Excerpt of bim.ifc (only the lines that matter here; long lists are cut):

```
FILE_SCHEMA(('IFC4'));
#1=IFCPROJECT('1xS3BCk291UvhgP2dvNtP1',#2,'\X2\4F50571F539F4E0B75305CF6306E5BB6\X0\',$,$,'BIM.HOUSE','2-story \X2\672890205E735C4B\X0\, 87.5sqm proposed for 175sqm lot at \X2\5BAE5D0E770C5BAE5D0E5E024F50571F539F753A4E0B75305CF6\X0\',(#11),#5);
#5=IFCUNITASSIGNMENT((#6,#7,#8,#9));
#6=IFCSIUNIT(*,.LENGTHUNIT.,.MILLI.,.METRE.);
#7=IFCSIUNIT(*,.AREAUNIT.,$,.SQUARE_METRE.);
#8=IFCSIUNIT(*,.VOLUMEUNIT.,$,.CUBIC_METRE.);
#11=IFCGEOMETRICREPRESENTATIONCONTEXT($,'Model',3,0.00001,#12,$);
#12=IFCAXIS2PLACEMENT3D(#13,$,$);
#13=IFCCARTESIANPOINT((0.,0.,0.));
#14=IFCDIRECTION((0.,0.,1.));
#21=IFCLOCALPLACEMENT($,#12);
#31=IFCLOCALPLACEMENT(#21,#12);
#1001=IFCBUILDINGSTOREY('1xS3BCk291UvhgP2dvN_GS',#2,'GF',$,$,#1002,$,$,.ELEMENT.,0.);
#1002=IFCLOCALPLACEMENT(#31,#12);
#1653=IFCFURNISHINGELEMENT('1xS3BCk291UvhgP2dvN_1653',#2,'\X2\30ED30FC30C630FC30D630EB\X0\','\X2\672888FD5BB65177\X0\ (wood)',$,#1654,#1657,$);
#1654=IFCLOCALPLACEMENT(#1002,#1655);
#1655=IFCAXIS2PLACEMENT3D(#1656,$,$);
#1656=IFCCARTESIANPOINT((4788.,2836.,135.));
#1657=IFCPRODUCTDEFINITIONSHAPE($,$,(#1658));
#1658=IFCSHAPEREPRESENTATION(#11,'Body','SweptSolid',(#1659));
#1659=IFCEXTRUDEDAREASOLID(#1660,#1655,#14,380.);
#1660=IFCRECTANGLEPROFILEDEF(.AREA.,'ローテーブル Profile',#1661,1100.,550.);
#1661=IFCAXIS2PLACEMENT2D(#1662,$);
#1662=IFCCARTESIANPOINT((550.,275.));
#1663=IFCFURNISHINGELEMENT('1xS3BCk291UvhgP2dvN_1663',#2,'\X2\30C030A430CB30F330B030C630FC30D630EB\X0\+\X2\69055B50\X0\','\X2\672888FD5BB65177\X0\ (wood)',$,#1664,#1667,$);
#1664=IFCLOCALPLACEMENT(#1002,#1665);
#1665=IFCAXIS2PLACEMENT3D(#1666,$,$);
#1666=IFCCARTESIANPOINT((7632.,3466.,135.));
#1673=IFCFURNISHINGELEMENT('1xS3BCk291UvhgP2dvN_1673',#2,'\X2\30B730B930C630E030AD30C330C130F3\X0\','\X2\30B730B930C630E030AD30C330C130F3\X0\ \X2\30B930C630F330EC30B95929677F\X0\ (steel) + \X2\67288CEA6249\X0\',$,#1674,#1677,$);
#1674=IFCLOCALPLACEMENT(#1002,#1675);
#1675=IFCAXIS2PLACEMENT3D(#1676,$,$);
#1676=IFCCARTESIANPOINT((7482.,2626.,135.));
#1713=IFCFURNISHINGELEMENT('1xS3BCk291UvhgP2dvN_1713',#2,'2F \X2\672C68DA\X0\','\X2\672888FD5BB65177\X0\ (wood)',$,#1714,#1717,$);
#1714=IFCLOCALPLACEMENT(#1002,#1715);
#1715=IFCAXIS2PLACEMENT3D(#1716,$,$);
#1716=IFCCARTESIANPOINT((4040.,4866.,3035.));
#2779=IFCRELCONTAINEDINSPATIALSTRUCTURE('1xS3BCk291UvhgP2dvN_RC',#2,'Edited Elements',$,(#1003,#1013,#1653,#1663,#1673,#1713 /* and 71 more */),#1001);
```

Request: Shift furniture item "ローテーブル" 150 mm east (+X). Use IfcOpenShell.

```python
import ifcopenshell
import ifcopenshell.api.geometry
import ifcopenshell.util.placement

model = ifcopenshell.open("bim.ifc")

item = model.by_guid("1xS3BCk291UvhgP2dvN_1653")
matrix = ifcopenshell.util.placement.get_local_placement(item.ObjectPlacement)
matrix[0, 3] += 150.0
ifcopenshell.api.geometry.edit_object_placement(model, product=item, matrix=matrix, is_si=False)

print(ifcopenshell.util.placement.get_local_placement(item.ObjectPlacement).round(3) + 0.0)

model.write("bim_updated.ifc")
```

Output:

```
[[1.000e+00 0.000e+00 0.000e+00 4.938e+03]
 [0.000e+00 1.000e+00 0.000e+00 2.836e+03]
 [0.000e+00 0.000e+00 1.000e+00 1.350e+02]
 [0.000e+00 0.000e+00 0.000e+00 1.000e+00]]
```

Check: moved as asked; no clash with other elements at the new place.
